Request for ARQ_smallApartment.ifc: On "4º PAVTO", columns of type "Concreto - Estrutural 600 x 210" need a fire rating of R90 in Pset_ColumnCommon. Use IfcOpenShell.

First a look at what the model holds.

```python
import ifcopenshell
import ifcopenshell.util.element

model = ifcopenshell.open("ARQ_smallApartment.ifc")
print(model.schema)
storey = next(s for s in model.by_type("IfcBuildingStorey") if s.Name == "4º PAVTO")
columns = [e for e in ifcopenshell.util.element.get_decomposition(storey) if e.is_a("IfcColumn")]
seen = {}
for e in columns:
    element_type = ifcopenshell.util.element.get_type(e)
    key = (element_type.Name if element_type != e and element_type else None, ifcopenshell.util.element.get_pset(e, "Pset_ColumnCommon", "FireRating"))
    seen[key] = seen.get(key, 0) + 1
for (name, value), count in sorted(seen.items(), key=str):
    print(count, "x", name, "|", value)
```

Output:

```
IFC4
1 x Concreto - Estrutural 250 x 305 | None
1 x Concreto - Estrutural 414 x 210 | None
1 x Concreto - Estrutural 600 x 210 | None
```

```python
import ifcopenshell
import ifcopenshell.api.pset
import ifcopenshell.util.element

model = ifcopenshell.open("ARQ_smallApartment.ifc")

storey = next(s for s in model.by_type("IfcBuildingStorey") if s.Name == "4º PAVTO")
columns = [e for e in ifcopenshell.util.element.get_decomposition(storey) if e.is_a("IfcColumn")]

count = 0
for e in columns:
    element_type = ifcopenshell.util.element.get_type(e)
    if element_type in (None, e) or element_type.Name != "Concreto - Estrutural 600 x 210":
        continue
    # add_pset returns the element's existing set when there is one.
    pset = ifcopenshell.api.pset.add_pset(model, product=e, name="Pset_ColumnCommon")
    ifcopenshell.api.pset.edit_pset(model, pset=pset, properties={"FireRating": "R90"})
    count += 1

print(count, "columns updated")

model.write("ARQ_smallApartment-out.ifc")
```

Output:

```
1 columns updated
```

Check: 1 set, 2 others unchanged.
